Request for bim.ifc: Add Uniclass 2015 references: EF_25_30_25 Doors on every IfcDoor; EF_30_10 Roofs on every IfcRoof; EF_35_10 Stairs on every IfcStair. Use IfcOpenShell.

First a look at what the model holds.

```python
import ifcopenshell

model = ifcopenshell.open("bim.ifc")
print(model.schema)
print("classifications:", [c.Name for c in model.by_type("IfcClassification")])
for ifc_class in ("IfcDoor", "IfcRoof", "IfcStair", "IfcWall", "IfcWindow"):
    print(ifc_class, len(model.by_type(ifc_class)))
```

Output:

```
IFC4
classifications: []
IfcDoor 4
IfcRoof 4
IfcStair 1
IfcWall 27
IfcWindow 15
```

```python
import ifcopenshell
import ifcopenshell.api.classification

model = ifcopenshell.open("bim.ifc")

system = ifcopenshell.api.classification.add_classification(model, classification="Uniclass 2015")

codes = {
    "IfcDoor": ("EF_25_30_25", "Doors"),
    "IfcRoof": ("EF_30_10", "Roofs"),
    "IfcStair": ("EF_35_10", "Stairs"),
}
for ifc_class, (code, name) in codes.items():
    products = model.by_type(ifc_class)
    ifcopenshell.api.classification.add_reference(
        model, products=products, classification=system, identification=code, name=name
    )
    print(code, len(products))

model.write("bim_edited.ifc")
```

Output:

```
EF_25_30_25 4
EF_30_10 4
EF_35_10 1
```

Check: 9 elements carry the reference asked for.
